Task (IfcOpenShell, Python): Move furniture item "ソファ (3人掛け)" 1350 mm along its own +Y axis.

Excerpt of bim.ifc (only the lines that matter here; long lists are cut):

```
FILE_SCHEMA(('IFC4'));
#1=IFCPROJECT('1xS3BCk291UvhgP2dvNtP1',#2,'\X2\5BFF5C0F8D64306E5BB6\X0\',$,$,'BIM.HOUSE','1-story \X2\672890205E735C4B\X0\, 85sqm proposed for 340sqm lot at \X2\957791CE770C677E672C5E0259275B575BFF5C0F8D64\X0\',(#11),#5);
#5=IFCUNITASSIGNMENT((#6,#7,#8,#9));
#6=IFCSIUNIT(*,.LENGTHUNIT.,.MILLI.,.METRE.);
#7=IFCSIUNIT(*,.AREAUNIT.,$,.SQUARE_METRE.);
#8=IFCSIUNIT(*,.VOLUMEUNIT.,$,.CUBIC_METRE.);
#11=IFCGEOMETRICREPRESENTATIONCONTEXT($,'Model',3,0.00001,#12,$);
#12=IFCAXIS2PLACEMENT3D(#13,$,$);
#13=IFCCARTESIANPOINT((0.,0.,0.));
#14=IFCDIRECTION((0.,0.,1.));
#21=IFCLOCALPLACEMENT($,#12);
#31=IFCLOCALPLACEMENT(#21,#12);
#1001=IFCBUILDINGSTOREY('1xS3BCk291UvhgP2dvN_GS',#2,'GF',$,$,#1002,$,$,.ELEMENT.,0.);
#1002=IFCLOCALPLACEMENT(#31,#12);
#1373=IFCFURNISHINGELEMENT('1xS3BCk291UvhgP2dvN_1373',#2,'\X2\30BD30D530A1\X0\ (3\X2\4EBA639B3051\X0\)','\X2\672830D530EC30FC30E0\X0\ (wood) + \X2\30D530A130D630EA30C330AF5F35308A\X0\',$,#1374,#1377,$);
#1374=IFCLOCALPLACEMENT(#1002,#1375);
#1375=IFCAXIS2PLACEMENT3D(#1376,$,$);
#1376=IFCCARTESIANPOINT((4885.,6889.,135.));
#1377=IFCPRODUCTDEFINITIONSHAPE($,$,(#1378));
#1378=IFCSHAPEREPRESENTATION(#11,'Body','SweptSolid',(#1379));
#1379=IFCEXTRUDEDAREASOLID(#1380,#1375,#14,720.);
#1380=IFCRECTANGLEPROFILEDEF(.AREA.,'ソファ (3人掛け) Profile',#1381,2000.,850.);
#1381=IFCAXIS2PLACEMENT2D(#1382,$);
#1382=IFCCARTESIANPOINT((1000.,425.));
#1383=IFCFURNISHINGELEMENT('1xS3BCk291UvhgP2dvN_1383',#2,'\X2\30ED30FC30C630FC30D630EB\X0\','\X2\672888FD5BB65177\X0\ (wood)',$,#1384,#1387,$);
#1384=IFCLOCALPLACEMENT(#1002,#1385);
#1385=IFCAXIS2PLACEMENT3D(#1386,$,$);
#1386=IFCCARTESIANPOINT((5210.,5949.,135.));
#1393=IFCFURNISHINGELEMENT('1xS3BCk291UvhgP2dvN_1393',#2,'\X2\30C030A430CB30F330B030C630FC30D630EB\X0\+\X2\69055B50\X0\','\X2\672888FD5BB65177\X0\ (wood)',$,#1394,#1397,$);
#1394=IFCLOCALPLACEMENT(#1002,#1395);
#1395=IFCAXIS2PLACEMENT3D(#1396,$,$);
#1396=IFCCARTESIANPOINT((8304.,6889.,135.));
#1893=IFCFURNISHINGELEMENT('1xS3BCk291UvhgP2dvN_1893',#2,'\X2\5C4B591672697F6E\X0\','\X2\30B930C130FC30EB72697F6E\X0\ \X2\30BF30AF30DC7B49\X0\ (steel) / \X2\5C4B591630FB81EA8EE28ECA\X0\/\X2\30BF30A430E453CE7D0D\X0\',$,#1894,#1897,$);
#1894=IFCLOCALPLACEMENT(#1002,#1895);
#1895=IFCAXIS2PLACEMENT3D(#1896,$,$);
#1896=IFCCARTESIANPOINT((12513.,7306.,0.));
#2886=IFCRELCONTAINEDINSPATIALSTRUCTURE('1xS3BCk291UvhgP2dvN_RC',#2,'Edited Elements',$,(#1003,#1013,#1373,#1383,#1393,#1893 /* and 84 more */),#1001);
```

```python
import ifcopenshell
import ifcopenshell.api.geometry
import ifcopenshell.util.placement
import ifcopenshell.util.unit

model = ifcopenshell.open("bim.ifc")
unit_scale = ifcopenshell.util.unit.calculate_unit_scale(model)

item = model.by_guid("1xS3BCk291UvhgP2dvN_1373")
matrix = ifcopenshell.util.placement.get_local_placement(item.ObjectPlacement)
matrix[:3, 3] += matrix[:3, 1] * 1.35 / unit_scale
ifcopenshell.api.geometry.edit_object_placement(model, product=item, matrix=matrix, is_si=False)

print(ifcopenshell.util.placement.get_local_placement(item.ObjectPlacement).round(3) + 0.0)

model.write("bim_updated.ifc")
```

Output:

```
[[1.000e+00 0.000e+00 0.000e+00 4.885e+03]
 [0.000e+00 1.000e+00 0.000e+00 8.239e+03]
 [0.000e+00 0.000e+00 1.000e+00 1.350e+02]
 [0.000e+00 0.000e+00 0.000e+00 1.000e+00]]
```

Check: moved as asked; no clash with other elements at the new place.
